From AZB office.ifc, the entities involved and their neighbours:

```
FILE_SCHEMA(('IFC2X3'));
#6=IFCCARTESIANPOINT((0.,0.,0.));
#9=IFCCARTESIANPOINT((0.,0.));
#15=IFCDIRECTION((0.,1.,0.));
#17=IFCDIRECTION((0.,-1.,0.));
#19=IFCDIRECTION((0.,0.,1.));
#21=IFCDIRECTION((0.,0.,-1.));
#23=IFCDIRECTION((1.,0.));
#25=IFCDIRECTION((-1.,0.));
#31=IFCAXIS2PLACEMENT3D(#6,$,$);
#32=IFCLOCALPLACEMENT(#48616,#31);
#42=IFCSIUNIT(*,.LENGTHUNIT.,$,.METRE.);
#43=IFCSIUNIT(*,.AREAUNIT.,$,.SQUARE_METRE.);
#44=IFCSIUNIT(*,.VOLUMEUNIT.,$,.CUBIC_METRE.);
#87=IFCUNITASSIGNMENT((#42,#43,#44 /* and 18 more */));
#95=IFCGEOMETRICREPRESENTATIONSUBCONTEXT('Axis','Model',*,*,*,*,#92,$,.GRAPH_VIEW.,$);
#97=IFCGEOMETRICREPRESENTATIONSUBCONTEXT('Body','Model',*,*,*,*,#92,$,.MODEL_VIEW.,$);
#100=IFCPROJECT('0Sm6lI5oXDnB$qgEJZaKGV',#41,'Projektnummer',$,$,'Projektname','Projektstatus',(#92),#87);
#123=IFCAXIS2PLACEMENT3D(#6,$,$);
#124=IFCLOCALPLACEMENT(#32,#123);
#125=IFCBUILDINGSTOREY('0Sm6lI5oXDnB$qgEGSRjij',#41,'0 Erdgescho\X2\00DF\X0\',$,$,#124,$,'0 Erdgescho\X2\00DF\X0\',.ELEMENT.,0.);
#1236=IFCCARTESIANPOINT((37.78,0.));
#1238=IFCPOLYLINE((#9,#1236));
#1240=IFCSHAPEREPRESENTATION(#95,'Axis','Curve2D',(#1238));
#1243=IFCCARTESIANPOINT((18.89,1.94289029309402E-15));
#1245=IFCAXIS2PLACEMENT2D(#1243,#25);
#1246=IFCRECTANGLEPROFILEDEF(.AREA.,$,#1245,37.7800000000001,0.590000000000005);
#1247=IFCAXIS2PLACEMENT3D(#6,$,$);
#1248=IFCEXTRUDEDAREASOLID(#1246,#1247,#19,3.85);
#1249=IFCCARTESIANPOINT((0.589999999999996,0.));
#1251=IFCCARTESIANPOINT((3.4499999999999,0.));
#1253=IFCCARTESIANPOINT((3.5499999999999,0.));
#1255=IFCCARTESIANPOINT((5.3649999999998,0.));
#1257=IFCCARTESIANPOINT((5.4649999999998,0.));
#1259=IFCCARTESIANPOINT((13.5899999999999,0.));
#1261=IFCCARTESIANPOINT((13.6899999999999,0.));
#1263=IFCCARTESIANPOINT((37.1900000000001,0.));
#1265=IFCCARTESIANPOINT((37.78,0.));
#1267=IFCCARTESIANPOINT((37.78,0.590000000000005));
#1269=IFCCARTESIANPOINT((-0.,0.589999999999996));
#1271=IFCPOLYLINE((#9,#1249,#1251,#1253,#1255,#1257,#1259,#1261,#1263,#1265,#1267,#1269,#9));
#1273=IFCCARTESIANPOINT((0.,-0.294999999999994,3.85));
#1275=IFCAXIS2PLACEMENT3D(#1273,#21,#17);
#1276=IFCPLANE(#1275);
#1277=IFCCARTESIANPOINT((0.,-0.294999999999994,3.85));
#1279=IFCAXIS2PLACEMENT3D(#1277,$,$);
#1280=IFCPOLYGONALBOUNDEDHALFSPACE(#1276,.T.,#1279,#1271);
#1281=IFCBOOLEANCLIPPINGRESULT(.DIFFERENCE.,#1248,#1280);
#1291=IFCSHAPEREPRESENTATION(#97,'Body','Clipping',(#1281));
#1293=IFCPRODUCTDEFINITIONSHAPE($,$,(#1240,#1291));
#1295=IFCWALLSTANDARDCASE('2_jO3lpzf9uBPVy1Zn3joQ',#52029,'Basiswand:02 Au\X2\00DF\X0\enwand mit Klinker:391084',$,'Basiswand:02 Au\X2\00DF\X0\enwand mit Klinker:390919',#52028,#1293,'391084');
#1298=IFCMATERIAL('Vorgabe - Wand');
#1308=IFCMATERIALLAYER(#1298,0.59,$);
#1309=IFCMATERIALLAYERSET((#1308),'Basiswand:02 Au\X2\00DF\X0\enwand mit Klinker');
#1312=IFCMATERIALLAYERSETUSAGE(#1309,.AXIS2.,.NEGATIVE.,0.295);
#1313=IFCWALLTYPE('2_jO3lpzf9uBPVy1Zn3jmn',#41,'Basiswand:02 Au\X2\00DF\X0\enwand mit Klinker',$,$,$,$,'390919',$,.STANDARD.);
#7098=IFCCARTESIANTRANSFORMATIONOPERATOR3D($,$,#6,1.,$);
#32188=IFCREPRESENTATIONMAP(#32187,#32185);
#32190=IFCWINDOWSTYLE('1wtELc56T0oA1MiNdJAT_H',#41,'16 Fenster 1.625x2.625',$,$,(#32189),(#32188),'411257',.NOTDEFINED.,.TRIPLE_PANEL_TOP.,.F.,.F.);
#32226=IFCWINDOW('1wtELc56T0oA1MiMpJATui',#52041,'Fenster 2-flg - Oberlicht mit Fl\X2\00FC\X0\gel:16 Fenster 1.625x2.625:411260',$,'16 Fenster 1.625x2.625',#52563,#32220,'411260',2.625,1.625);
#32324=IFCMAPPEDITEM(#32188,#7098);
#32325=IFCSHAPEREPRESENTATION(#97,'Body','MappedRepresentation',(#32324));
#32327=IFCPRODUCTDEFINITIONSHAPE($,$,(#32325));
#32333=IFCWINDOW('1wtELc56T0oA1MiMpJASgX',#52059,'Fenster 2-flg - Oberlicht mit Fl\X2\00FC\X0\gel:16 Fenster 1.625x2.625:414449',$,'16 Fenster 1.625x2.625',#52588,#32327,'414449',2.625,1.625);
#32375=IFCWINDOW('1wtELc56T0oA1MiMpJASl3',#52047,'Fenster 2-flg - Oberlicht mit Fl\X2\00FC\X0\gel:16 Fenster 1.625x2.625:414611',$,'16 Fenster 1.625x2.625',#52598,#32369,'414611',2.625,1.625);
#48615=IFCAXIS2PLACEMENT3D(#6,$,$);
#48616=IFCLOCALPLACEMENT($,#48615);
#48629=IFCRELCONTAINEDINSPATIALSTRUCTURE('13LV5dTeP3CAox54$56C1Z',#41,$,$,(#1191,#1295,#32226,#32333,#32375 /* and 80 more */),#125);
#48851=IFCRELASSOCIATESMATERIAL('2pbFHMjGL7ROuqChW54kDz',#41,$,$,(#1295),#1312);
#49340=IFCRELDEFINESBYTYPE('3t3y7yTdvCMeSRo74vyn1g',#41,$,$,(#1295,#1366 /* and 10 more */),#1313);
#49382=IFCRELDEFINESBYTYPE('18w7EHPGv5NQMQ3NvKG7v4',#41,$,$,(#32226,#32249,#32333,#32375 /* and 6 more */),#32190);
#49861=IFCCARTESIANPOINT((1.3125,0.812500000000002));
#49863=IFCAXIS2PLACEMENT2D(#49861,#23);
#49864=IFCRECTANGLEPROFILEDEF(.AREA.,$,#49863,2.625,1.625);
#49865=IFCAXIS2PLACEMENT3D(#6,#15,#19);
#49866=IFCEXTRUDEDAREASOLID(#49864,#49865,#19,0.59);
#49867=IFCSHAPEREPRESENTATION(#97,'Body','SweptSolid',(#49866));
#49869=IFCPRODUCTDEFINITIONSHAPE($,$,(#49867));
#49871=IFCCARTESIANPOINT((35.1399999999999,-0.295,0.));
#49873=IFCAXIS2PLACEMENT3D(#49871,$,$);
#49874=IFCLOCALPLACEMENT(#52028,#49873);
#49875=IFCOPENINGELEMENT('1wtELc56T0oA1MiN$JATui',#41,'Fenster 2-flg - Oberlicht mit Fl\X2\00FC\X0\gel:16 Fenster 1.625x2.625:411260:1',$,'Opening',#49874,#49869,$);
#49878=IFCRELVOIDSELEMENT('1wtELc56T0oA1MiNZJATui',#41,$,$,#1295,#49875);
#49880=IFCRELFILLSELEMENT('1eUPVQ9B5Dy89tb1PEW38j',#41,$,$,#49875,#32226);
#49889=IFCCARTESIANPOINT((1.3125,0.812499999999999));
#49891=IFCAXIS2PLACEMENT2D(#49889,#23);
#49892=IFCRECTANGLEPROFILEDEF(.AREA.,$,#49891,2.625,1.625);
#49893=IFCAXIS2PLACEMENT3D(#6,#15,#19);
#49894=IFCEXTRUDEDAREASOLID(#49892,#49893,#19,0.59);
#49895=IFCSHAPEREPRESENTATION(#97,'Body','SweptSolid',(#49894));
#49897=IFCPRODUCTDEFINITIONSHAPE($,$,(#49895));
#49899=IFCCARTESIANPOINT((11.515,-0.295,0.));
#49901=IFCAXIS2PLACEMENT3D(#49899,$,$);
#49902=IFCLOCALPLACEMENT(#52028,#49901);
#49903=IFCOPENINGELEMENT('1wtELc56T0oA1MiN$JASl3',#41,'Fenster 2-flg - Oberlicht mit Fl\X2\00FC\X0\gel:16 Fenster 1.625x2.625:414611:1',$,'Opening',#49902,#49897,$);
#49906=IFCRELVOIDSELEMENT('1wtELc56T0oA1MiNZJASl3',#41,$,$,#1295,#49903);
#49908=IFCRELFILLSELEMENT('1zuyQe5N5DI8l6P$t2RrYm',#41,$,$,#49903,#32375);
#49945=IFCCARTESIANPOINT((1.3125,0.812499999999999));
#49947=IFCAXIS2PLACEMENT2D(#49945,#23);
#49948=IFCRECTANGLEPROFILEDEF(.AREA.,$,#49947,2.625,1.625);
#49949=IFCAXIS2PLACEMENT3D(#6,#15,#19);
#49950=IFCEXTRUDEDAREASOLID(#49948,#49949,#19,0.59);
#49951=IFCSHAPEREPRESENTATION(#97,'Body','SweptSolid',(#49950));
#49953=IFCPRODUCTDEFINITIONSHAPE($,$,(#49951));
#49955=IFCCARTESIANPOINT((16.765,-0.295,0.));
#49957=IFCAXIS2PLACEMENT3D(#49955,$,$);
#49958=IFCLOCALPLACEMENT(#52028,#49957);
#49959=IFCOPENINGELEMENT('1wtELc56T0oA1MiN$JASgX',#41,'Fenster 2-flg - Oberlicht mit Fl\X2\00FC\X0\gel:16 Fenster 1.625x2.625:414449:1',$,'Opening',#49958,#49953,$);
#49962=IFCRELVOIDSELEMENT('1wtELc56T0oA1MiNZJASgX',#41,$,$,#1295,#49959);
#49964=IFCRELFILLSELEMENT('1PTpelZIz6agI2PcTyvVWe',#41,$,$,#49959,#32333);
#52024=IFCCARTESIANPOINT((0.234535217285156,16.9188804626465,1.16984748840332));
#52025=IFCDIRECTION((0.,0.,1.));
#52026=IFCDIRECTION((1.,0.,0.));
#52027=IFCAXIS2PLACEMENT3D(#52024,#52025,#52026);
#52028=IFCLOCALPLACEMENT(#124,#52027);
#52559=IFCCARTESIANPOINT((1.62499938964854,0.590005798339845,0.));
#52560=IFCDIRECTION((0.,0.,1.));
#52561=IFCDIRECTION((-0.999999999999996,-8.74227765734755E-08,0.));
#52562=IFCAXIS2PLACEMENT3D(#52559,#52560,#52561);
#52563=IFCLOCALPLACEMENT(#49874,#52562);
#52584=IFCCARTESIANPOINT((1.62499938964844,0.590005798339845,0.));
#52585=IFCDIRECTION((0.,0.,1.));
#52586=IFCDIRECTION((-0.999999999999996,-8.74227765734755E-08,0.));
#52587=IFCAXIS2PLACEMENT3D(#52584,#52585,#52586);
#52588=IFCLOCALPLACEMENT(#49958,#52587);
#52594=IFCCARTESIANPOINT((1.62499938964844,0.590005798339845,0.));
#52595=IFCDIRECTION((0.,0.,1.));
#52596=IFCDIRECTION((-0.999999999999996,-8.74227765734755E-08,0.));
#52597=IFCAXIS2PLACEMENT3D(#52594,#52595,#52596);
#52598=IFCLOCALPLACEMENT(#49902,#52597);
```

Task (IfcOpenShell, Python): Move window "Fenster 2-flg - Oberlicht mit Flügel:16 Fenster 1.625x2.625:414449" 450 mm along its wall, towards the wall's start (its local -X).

```python
import ifcopenshell
import ifcopenshell.api.geometry
import ifcopenshell.util.placement
import ifcopenshell.util.unit

model = ifcopenshell.open("AZB office.ifc")
unit_scale = ifcopenshell.util.unit.calculate_unit_scale(model)

window = model.by_guid("1wtELc56T0oA1MiMpJASgX")
opening = window.FillsVoids[0].RelatingOpeningElement
wall = opening.VoidsElements[0].RelatingBuildingElement

wall_matrix = ifcopenshell.util.placement.get_local_placement(wall.ObjectPlacement)
shift = wall_matrix[:3, 0] * -0.45 / unit_scale
before = ifcopenshell.util.placement.get_local_placement(window.ObjectPlacement)[:3, 3].copy()

# The window is placed relative to its opening, so it follows when the opening moves.
matrix = ifcopenshell.util.placement.get_local_placement(opening.ObjectPlacement)
matrix[:3, 3] += shift
ifcopenshell.api.geometry.edit_object_placement(
    model, product=opening, matrix=matrix, is_si=False, should_transform_children=True
)

after = ifcopenshell.util.placement.get_local_placement(window.ObjectPlacement)[:3, 3]
print("window moved by", (after - before).round(3) + 0.0)

model.write("AZB office_rev.ifc")
```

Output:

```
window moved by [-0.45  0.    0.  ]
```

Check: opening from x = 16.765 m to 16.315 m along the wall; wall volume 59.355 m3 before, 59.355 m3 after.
